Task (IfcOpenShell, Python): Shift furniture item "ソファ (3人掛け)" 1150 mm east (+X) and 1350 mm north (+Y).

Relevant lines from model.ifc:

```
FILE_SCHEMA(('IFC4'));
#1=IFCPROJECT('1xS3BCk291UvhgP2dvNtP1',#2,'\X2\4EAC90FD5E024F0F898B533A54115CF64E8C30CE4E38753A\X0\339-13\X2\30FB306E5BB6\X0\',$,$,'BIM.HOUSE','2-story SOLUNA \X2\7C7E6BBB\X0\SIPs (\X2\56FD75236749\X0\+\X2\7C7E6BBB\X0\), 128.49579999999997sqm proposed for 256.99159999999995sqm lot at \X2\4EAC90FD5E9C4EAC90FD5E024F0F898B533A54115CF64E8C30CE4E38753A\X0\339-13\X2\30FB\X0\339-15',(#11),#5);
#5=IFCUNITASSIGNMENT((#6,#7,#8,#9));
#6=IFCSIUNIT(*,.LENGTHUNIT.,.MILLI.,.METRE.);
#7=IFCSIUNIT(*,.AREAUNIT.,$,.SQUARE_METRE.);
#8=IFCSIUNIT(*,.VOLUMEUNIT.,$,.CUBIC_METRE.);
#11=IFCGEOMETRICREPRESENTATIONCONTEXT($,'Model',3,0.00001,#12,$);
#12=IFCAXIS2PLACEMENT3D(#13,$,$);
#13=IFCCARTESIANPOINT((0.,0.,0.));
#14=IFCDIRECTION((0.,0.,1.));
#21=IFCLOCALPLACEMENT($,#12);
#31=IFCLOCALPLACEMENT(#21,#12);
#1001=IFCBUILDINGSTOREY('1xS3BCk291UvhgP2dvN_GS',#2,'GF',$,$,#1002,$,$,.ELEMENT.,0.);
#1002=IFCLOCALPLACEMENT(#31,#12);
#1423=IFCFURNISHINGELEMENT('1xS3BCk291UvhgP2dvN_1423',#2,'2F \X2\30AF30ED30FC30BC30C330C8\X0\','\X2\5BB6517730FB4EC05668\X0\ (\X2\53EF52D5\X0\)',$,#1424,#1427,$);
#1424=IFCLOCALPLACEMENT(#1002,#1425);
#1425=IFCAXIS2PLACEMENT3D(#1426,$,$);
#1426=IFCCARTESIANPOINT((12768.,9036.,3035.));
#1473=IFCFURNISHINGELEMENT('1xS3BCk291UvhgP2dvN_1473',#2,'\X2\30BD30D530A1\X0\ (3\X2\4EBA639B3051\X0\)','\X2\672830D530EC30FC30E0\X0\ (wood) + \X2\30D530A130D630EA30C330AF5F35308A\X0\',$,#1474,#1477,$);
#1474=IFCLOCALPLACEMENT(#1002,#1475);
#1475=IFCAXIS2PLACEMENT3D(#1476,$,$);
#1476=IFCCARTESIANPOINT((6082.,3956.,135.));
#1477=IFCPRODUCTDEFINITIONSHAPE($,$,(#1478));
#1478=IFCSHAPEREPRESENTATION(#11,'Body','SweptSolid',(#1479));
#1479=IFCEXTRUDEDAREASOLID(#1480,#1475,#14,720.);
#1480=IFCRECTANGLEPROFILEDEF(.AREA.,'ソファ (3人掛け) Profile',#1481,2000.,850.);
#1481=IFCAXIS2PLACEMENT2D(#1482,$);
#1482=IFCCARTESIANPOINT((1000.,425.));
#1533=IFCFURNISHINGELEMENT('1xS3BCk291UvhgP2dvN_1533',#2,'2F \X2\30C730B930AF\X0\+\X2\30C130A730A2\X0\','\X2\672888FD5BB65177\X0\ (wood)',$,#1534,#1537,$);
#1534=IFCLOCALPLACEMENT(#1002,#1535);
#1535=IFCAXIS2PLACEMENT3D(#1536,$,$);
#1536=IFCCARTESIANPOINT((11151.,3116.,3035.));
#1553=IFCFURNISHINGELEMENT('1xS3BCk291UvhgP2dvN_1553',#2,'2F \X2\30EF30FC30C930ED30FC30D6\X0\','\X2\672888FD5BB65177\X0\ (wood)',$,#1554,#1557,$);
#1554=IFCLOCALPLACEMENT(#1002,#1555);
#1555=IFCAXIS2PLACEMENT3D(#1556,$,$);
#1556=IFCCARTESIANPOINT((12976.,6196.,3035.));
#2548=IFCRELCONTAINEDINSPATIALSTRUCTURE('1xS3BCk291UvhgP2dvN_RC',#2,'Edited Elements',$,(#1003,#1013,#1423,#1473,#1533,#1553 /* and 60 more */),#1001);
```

```python
import ifcopenshell
import ifcopenshell.api.geometry
import ifcopenshell.util.placement
import ifcopenshell.util.unit

model = ifcopenshell.open("model.ifc")
unit_scale = ifcopenshell.util.unit.calculate_unit_scale(model)

item = model.by_guid("1xS3BCk291UvhgP2dvN_1473")
matrix = ifcopenshell.util.placement.get_local_placement(item.ObjectPlacement)
matrix[0, 3] += 1.15 / unit_scale
matrix[1, 3] += 1.35 / unit_scale
ifcopenshell.api.geometry.edit_object_placement(model, product=item, matrix=matrix, is_si=False)

print(ifcopenshell.util.placement.get_local_placement(item.ObjectPlacement).round(3) + 0.0)

model.write("model_rev.ifc")
```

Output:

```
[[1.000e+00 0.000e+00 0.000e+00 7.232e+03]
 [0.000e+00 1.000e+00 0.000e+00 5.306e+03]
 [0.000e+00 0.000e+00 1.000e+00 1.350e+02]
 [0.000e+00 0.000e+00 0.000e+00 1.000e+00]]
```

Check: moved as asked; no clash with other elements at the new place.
